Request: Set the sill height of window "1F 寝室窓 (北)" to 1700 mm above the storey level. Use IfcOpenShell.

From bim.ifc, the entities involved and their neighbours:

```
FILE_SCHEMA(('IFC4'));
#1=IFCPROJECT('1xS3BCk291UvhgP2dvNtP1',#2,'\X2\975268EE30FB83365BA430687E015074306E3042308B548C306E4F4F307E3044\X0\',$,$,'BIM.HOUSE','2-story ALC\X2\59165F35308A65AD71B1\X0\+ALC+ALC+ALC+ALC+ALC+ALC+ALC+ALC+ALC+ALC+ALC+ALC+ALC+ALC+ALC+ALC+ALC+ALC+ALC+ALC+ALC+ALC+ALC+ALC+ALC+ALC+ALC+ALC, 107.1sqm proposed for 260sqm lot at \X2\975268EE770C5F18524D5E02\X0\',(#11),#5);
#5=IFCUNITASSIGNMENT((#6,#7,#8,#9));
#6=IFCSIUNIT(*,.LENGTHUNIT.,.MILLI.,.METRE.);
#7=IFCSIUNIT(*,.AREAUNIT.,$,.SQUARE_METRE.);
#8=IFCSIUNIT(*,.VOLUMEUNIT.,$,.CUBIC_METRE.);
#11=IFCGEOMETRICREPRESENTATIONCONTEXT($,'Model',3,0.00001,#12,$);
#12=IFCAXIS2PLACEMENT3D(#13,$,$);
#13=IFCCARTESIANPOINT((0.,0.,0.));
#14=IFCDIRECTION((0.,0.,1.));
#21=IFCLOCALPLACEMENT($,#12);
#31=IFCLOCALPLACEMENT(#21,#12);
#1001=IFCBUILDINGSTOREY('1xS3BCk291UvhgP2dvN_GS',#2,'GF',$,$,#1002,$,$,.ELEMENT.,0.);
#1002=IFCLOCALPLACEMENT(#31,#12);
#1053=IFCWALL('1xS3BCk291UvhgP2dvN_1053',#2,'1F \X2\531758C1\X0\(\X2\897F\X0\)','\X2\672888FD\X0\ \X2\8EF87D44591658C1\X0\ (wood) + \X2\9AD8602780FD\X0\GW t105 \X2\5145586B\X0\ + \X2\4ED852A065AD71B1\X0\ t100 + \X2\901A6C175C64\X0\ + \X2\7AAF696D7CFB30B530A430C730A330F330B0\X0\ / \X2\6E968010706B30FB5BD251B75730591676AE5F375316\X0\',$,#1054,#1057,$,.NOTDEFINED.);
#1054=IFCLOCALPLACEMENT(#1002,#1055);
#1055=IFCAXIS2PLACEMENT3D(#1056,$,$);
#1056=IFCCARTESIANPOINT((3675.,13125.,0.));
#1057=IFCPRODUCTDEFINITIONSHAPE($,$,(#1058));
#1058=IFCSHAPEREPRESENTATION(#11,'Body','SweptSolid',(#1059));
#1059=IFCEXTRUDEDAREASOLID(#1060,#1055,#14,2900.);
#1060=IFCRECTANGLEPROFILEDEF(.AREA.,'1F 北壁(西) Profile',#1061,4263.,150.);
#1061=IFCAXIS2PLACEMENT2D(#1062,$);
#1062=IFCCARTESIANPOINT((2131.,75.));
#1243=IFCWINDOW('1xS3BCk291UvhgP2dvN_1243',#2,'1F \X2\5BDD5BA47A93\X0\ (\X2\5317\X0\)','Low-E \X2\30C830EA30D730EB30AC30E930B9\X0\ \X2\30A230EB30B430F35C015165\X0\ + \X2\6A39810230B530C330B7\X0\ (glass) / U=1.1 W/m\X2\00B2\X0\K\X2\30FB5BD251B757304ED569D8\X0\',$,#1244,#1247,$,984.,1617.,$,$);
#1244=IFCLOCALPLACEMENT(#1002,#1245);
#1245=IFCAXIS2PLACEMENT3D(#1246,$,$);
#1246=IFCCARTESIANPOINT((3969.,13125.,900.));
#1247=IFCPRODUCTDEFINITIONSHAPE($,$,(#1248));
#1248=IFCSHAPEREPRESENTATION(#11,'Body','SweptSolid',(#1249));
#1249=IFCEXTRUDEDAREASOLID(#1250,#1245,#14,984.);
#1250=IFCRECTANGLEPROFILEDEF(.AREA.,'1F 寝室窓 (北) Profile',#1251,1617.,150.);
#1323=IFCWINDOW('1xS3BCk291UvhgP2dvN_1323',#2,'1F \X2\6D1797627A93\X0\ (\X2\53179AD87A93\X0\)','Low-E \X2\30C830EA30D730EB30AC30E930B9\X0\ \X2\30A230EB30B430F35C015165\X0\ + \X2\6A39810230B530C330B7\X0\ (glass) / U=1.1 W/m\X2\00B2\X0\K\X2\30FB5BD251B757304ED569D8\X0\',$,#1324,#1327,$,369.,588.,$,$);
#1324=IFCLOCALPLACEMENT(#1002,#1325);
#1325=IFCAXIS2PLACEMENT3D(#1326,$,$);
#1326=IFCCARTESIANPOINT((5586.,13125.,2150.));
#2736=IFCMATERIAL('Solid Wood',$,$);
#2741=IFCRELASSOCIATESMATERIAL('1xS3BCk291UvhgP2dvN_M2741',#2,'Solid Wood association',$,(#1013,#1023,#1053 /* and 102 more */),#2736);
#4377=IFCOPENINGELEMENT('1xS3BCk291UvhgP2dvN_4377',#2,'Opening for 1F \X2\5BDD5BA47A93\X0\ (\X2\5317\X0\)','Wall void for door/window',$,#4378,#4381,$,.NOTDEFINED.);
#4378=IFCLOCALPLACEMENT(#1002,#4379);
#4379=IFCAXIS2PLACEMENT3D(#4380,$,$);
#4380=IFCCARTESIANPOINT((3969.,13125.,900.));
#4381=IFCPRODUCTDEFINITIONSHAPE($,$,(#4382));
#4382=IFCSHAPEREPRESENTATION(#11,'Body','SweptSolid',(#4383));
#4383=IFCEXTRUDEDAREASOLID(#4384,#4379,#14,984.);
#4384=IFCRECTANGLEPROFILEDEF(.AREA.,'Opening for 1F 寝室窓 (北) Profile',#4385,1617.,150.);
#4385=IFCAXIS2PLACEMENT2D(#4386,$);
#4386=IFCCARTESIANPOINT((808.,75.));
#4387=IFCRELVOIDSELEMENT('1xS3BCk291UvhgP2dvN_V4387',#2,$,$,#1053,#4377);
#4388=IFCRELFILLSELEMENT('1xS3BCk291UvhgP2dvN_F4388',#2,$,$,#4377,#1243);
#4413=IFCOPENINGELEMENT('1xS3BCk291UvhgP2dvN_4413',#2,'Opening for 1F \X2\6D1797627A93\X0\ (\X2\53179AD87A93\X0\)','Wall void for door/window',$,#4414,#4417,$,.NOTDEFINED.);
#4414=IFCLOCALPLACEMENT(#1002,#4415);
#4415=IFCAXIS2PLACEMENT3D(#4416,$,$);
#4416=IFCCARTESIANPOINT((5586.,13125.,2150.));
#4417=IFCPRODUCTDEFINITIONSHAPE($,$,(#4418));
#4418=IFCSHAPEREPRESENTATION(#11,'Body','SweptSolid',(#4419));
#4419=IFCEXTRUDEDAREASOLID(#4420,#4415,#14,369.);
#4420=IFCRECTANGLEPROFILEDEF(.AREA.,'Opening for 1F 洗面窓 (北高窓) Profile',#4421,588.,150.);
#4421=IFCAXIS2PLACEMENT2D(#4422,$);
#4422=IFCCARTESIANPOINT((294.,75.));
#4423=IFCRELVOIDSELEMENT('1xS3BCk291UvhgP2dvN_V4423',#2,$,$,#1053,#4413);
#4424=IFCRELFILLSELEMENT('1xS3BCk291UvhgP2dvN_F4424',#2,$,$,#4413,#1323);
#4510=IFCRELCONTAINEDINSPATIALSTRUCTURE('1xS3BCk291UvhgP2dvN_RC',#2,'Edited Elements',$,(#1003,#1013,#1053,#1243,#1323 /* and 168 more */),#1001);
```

```python
import numpy as np
import ifcopenshell
import ifcopenshell.api.geometry
import ifcopenshell.geom
import ifcopenshell.util.element
import ifcopenshell.util.placement
import ifcopenshell.util.shape
import ifcopenshell.util.unit

model = ifcopenshell.open("bim.ifc")
unit_scale = ifcopenshell.util.unit.calculate_unit_scale(model)

window = model.by_guid("1xS3BCk291UvhgP2dvN_1243")
opening = window.FillsVoids[0].RelatingOpeningElement
storey = ifcopenshell.util.element.get_container(window, ifc_class="IfcBuildingStorey")
level = ifcopenshell.util.placement.get_local_placement(storey.ObjectPlacement)[2, 3]

# The opening's origin need not be at the sill, so measure its lowest point.
shape = ifcopenshell.geom.create_shape(ifcopenshell.geom.settings(), opening)
bottom = ifcopenshell.util.shape.get_shape_bottom_elevation(shape, shape.geometry) / unit_scale
dz = level + 1.7 / unit_scale - bottom

shift = np.array([0.0, 0.0, dz])
# The window is not placed relative to its opening, so move both.
for product in (opening, window):
    matrix = ifcopenshell.util.placement.get_local_placement(product.ObjectPlacement)
    matrix[:3, 3] += shift
    ifcopenshell.api.geometry.edit_object_placement(model, product=product, matrix=matrix, is_si=False)

print(f"moved by {dz * unit_scale:+.3f} m")

model.write("bim_v2.ifc")
```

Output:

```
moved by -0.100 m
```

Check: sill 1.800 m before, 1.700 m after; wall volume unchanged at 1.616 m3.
